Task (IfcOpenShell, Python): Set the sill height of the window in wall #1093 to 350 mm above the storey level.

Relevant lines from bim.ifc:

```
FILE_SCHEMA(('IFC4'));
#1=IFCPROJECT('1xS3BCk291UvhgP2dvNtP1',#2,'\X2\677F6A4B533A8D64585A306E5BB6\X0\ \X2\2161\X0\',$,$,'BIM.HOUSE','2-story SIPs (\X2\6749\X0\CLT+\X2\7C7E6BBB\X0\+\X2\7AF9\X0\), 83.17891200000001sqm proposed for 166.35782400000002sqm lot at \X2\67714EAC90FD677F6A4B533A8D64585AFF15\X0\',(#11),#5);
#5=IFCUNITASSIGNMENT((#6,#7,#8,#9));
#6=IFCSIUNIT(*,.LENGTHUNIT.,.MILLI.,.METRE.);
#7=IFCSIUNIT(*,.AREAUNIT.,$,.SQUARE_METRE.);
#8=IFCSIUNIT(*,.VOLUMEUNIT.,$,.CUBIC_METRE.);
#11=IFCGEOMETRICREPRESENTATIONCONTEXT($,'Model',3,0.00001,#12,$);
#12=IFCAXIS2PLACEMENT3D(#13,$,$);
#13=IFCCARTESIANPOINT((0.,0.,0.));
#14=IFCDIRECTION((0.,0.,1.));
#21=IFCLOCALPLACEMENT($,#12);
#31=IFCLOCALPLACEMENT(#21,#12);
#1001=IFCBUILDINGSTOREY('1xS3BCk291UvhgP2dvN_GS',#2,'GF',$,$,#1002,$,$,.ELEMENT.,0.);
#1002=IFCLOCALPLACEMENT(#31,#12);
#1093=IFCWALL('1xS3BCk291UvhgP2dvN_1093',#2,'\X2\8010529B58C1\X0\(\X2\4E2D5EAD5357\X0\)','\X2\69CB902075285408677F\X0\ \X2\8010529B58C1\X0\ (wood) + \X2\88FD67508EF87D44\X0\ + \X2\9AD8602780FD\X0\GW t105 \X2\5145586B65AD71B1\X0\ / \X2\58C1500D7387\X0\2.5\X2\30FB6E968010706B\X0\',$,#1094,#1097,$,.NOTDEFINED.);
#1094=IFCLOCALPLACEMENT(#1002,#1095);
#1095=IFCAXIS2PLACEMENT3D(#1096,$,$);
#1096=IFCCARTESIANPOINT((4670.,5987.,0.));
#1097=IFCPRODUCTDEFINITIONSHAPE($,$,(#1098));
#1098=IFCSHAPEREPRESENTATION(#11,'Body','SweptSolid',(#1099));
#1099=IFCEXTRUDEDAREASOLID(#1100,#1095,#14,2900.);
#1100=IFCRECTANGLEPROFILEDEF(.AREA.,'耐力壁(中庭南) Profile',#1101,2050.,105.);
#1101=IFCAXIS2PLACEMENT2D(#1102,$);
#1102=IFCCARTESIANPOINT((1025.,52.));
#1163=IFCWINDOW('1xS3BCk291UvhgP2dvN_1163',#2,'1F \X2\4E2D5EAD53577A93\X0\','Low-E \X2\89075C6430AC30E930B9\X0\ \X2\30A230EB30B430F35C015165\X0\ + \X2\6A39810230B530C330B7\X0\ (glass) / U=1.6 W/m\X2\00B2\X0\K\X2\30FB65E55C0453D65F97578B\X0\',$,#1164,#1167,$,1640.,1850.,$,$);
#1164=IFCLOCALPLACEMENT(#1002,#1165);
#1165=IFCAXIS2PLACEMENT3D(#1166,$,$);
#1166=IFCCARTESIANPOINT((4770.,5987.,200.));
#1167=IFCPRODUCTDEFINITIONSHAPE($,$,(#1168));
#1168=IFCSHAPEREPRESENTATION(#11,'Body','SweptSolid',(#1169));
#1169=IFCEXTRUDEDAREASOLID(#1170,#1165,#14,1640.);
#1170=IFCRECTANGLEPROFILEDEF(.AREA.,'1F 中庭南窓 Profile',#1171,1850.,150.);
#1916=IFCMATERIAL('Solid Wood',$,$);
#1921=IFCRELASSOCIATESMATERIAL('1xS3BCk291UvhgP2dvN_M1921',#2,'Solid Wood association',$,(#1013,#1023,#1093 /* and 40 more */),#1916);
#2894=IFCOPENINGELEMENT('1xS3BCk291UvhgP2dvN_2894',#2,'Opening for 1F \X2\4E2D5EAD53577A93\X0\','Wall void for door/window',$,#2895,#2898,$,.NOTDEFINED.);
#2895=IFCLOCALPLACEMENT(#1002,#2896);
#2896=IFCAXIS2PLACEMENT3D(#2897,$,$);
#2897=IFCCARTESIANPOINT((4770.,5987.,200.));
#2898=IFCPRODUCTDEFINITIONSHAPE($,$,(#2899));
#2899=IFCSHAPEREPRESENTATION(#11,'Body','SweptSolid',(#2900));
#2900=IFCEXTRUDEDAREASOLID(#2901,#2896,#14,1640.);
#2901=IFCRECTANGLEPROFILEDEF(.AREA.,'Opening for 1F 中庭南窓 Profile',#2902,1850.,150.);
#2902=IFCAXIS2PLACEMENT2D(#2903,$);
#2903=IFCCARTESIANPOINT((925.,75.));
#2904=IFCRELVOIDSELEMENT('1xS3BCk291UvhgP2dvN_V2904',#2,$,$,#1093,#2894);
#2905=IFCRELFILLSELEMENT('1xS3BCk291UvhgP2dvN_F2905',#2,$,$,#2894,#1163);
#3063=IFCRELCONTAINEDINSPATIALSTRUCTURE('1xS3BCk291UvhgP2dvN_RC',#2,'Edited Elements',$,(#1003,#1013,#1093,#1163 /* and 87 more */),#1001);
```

```python
import numpy as np
import ifcopenshell
import ifcopenshell.api.geometry
import ifcopenshell.geom
import ifcopenshell.util.element
import ifcopenshell.util.placement
import ifcopenshell.util.shape
import ifcopenshell.util.unit

model = ifcopenshell.open("bim.ifc")
unit_scale = ifcopenshell.util.unit.calculate_unit_scale(model)

window = model.by_guid("1xS3BCk291UvhgP2dvN_1163")
opening = window.FillsVoids[0].RelatingOpeningElement
storey = ifcopenshell.util.element.get_container(window, ifc_class="IfcBuildingStorey")
level = ifcopenshell.util.placement.get_local_placement(storey.ObjectPlacement)[2, 3]

# The opening's origin need not be at the sill, so measure its lowest point.
shape = ifcopenshell.geom.create_shape(ifcopenshell.geom.settings(), opening)
bottom = ifcopenshell.util.shape.get_shape_bottom_elevation(shape, shape.geometry) / unit_scale
dz = level + 0.35 / unit_scale - bottom

shift = np.array([0.0, 0.0, dz])
# The window is not placed relative to its opening, so move both.
for product in (opening, window):
    matrix = ifcopenshell.util.placement.get_local_placement(product.ObjectPlacement)
    matrix[:3, 3] += shift
    ifcopenshell.api.geometry.edit_object_placement(model, product=product, matrix=matrix, is_si=False)

print(f"moved by {dz * unit_scale:+.3f} m")

model.write("bim_v2.ifc")
```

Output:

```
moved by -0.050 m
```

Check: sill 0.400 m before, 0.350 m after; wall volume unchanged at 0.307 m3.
